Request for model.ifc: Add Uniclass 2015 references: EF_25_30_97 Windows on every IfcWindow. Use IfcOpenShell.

First a look at what the model holds.

```python
import ifcopenshell

model = ifcopenshell.open("model.ifc")
print(model.schema)
print("classifications:", [c.Name for c in model.by_type("IfcClassification")])
for ifc_class in ("IfcDoor", "IfcRoof", "IfcStair", "IfcWall", "IfcWindow"):
    print(ifc_class, len(model.by_type(ifc_class)))
```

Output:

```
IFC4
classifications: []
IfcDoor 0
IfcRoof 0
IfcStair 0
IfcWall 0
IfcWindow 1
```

```python
import ifcopenshell
import ifcopenshell.api.classification

model = ifcopenshell.open("model.ifc")

system = ifcopenshell.api.classification.add_classification(model, classification="Uniclass 2015")

codes = {
    "IfcWindow": ("EF_25_30_97", "Windows"),
}
for ifc_class, (code, name) in codes.items():
    products = model.by_type(ifc_class)
    ifcopenshell.api.classification.add_reference(
        model, products=products, classification=system, identification=code, name=name
    )
    print(code, len(products))

model.write("model_updated.ifc")
```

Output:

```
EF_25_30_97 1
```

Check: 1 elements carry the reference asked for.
